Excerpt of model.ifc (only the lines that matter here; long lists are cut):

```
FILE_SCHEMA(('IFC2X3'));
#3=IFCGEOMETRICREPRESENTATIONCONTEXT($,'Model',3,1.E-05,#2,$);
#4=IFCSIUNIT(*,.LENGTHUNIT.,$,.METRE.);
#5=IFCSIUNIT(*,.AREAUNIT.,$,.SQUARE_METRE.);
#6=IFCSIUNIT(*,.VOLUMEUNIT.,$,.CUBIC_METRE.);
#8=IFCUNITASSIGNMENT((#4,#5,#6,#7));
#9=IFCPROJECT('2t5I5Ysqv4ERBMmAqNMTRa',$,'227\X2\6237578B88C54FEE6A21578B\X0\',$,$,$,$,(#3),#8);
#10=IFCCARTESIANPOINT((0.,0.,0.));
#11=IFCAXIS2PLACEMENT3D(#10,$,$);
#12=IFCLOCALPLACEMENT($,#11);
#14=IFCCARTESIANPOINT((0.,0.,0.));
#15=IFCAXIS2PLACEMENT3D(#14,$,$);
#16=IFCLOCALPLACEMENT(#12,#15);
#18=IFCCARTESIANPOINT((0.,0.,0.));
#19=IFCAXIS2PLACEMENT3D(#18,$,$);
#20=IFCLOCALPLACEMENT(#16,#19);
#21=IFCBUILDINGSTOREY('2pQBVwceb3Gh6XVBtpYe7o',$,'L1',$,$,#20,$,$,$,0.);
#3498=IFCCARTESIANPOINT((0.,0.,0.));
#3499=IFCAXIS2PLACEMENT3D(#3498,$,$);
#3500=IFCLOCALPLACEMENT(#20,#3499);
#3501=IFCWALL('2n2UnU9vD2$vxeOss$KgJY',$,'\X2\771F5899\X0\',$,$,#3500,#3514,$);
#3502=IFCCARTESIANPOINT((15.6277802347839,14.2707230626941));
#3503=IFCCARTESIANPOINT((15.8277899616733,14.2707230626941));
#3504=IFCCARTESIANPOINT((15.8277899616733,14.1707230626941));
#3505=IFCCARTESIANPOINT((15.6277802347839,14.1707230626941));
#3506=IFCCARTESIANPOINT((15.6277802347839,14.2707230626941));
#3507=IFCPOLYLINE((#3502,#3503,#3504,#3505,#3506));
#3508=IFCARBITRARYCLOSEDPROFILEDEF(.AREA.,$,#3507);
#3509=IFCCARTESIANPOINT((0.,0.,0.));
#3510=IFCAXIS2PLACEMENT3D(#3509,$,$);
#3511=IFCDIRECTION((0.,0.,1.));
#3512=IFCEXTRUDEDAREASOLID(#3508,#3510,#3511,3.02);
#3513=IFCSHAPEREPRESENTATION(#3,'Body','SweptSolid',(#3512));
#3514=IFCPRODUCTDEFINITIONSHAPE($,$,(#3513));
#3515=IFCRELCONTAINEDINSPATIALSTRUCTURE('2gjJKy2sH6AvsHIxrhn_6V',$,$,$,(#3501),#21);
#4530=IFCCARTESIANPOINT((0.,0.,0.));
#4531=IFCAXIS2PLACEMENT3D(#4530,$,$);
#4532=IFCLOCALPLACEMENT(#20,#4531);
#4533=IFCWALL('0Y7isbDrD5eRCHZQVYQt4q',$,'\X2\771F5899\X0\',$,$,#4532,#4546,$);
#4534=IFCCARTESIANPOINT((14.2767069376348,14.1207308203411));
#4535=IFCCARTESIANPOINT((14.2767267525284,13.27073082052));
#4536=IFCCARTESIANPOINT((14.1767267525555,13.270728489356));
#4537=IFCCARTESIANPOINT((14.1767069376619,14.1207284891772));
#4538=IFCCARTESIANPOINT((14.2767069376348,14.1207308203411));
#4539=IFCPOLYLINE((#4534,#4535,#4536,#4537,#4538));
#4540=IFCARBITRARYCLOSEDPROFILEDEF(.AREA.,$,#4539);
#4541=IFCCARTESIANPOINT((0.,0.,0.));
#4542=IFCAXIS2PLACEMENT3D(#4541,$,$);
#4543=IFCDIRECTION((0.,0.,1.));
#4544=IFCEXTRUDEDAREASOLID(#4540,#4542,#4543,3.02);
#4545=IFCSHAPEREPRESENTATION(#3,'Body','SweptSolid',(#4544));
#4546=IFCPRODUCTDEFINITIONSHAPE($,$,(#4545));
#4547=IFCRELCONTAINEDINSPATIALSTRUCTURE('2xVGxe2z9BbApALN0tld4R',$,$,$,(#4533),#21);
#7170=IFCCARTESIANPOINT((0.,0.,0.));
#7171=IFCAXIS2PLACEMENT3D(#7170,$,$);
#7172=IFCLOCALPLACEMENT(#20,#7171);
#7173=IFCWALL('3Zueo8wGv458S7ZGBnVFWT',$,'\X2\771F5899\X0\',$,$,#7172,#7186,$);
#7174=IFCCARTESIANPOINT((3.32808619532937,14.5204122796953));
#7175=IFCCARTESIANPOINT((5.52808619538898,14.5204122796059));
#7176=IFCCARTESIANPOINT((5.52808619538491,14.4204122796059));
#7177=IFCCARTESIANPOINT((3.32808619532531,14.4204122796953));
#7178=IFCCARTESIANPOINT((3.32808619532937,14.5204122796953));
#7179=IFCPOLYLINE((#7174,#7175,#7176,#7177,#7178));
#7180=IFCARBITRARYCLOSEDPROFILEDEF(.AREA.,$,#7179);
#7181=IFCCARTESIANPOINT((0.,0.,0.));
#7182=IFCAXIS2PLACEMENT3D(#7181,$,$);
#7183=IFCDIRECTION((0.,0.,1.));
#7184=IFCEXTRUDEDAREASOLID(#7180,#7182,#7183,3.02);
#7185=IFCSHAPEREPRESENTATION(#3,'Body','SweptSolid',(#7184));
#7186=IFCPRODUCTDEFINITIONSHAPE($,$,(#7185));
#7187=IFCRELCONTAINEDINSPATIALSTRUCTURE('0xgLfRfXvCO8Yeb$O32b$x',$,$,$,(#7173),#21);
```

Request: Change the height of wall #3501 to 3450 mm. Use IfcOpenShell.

```python
import ifcopenshell
import ifcopenshell.geom
import ifcopenshell.util.shape
import ifcopenshell.util.unit

model = ifcopenshell.open("model.ifc")
unit_scale = ifcopenshell.util.unit.calculate_unit_scale(model)
settings = ifcopenshell.geom.settings()


def volume(element):
    """Net volume in cubic metres, openings subtracted."""
    shape = ifcopenshell.geom.create_shape(settings, element)
    return ifcopenshell.util.shape.get_volume(shape.geometry)


wall = model.by_id(3501)
before = volume(wall)

body = next(r for r in wall.Representation.Representations if r.RepresentationIdentifier == "Body")
solid = body.Items[0]
old_height = solid.Depth
solid.Depth = 3.45 / unit_scale
after = volume(wall)

print(f"height {old_height:g} -> {solid.Depth:g}, volume {before:.3f} -> {after:.3f} m3")

model.write("model_updated.ifc")
```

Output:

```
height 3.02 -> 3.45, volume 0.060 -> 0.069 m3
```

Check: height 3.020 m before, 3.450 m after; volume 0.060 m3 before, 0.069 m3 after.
